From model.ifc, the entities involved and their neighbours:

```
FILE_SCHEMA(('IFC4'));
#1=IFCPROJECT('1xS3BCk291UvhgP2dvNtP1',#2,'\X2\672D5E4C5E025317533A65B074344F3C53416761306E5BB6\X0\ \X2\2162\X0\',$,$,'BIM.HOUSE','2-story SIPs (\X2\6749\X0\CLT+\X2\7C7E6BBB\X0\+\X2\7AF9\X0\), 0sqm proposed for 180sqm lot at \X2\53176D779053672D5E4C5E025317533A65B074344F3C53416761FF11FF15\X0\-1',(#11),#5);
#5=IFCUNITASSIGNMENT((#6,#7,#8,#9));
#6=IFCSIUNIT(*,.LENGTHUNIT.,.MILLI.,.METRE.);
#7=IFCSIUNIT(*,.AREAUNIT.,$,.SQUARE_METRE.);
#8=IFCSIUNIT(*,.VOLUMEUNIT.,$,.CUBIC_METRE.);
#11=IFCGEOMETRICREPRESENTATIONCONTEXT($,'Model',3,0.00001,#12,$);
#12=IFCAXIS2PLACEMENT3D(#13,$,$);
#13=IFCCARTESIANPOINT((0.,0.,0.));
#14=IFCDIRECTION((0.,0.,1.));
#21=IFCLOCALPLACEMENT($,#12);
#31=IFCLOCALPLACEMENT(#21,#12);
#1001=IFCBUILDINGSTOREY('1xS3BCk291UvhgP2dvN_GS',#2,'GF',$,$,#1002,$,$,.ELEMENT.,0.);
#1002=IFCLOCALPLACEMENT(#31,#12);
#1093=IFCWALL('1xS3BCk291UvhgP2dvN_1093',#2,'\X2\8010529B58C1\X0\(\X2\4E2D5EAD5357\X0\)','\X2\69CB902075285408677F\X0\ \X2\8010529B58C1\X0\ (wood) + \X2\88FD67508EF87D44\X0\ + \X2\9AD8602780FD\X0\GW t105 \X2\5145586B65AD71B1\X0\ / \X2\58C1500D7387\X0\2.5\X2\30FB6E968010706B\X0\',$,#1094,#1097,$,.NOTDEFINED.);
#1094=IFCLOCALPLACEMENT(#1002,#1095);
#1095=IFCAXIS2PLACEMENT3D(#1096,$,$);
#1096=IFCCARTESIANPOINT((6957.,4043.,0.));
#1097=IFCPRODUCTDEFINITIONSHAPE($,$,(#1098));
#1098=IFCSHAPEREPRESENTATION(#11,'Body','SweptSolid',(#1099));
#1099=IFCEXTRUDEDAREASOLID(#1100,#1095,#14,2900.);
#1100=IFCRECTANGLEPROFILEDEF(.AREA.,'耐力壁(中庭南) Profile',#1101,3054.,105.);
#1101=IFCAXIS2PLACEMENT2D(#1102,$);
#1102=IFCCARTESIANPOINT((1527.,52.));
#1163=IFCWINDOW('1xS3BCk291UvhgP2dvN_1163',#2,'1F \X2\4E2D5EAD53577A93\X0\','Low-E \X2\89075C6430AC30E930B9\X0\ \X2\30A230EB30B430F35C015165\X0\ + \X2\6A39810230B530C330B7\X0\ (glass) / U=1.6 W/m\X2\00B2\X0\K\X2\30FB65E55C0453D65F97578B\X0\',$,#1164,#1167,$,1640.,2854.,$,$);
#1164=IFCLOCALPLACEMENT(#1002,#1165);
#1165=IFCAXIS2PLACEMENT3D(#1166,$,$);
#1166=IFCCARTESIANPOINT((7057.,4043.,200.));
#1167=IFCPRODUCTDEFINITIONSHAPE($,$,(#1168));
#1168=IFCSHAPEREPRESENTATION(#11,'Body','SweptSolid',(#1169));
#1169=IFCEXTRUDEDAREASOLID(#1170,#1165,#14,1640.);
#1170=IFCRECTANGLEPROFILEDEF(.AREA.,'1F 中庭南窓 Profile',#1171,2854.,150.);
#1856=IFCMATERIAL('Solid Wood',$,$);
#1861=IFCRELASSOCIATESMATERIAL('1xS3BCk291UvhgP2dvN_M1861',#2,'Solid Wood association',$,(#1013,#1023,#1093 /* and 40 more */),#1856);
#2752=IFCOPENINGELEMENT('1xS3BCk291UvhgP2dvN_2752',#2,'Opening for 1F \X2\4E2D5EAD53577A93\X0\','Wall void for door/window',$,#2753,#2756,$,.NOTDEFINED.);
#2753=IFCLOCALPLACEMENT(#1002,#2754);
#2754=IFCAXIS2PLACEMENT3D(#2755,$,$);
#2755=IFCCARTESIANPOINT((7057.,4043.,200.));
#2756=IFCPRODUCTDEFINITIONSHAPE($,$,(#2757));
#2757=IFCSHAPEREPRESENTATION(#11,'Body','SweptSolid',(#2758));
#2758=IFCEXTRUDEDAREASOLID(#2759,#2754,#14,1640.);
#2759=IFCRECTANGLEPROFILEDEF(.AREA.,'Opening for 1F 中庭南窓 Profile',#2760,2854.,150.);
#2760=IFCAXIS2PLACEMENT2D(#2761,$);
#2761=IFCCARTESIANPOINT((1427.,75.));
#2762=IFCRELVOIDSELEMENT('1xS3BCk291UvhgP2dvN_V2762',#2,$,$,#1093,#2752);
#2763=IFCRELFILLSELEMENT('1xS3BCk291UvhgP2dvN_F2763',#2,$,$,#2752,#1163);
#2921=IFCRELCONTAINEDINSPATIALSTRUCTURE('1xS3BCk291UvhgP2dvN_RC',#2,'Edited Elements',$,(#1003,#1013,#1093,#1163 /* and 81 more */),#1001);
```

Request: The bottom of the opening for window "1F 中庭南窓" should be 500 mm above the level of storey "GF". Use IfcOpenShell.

```python
import numpy as np
import ifcopenshell
import ifcopenshell.api.geometry
import ifcopenshell.geom
import ifcopenshell.util.element
import ifcopenshell.util.placement
import ifcopenshell.util.shape
import ifcopenshell.util.unit

model = ifcopenshell.open("model.ifc")
unit_scale = ifcopenshell.util.unit.calculate_unit_scale(model)

window = model.by_guid("1xS3BCk291UvhgP2dvN_1163")
opening = window.FillsVoids[0].RelatingOpeningElement
storey = ifcopenshell.util.element.get_container(window, ifc_class="IfcBuildingStorey")
level = ifcopenshell.util.placement.get_local_placement(storey.ObjectPlacement)[2, 3]

# The opening's origin need not be at the sill, so measure its lowest point.
shape = ifcopenshell.geom.create_shape(ifcopenshell.geom.settings(), opening)
bottom = ifcopenshell.util.shape.get_shape_bottom_elevation(shape, shape.geometry) / unit_scale
dz = level + 0.5 / unit_scale - bottom

shift = np.array([0.0, 0.0, dz])
# The window is not placed relative to its opening, so move both.
for product in (opening, window):
    matrix = ifcopenshell.util.placement.get_local_placement(product.ObjectPlacement)
    matrix[:3, 3] += shift
    ifcopenshell.api.geometry.edit_object_placement(model, product=product, matrix=matrix, is_si=False)

print(f"moved by {dz * unit_scale:+.3f} m")

model.write("model_updated.ifc")
```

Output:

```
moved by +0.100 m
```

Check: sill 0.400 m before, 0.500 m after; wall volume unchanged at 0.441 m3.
